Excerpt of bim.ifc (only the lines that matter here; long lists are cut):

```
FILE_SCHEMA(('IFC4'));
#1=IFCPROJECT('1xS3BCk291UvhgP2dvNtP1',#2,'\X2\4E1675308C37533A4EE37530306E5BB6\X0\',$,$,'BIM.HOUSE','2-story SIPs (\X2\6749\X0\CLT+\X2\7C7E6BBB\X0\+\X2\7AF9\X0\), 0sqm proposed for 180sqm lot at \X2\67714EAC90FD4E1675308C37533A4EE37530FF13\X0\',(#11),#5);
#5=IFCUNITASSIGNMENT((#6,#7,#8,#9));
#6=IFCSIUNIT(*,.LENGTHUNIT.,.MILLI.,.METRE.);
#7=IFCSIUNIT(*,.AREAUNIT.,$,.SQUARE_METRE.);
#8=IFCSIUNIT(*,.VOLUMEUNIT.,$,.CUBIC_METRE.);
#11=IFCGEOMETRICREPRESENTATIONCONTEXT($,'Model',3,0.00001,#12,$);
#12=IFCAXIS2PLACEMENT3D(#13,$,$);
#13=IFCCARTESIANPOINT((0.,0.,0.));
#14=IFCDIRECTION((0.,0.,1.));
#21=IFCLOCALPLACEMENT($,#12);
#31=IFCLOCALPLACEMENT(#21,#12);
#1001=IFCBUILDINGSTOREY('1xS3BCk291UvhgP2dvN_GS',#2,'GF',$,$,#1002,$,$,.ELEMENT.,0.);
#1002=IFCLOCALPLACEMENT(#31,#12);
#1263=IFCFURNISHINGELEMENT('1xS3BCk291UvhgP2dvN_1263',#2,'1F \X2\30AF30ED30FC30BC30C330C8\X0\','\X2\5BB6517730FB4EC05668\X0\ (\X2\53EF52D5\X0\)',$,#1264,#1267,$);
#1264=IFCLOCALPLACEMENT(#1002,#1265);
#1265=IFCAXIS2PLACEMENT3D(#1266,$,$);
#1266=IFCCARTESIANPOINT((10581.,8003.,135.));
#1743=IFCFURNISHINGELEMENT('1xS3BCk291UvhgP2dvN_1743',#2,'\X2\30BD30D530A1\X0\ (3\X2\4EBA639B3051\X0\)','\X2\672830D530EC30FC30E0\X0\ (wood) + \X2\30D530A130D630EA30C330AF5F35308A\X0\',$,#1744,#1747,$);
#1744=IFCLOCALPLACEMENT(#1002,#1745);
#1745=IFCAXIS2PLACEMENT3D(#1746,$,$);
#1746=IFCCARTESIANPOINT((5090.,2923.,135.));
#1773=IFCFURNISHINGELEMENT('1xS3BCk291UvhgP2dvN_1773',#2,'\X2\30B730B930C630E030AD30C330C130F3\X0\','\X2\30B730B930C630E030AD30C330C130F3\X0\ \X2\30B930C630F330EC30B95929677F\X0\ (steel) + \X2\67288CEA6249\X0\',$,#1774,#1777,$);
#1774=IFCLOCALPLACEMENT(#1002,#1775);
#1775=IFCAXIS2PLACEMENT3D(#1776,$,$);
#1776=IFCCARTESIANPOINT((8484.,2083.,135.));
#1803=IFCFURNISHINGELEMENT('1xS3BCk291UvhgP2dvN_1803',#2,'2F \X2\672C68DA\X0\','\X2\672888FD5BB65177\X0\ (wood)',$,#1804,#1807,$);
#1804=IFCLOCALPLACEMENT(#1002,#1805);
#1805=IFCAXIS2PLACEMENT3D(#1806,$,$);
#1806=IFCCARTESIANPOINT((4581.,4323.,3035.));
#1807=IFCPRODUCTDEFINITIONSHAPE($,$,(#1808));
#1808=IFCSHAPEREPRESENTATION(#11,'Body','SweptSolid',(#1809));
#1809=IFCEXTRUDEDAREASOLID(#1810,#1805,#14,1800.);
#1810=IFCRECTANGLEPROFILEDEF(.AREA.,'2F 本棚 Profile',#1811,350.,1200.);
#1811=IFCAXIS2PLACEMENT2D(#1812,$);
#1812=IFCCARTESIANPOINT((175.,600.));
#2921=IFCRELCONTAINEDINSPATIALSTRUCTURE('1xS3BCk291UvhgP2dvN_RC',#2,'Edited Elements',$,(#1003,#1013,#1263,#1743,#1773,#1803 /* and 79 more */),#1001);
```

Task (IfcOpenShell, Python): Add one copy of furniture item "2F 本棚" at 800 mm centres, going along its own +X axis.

```python
import ifcopenshell
import ifcopenshell.api.geometry
import ifcopenshell.api.root
import ifcopenshell.util.element
import ifcopenshell.util.placement

model = ifcopenshell.open("bim.ifc")


def reuse_history(source, copy):
    """copy_class also copies each property set's owner history, people and application; keep the originals."""
    for rel in copy.IsDefinedBy:
        if rel.is_a("IfcRelDefinesByProperties") and (history := rel.RelatingPropertyDefinition.OwnerHistory):
            rel.RelatingPropertyDefinition.OwnerHistory = source.OwnerHistory
            ifcopenshell.util.element.remove_deep2(model, history)


source = model.by_id(1803)
base = ifcopenshell.util.placement.get_local_placement(source.ObjectPlacement)
step = base[:3, 0] * 800.0

for i in range(1, 2):
    copy = ifcopenshell.api.root.copy_class(model, product=source)
    copy.Representation = ifcopenshell.util.element.copy_deep(
        model, source.Representation, exclude=["IfcGeometricRepresentationContext", "IfcRepresentationMap"]
    )
    reuse_history(source, copy)
    matrix = base.copy()
    matrix[:3, 3] += i * step
    print("added at", matrix[:3, 3].round(3) + 0.0)
    ifcopenshell.api.geometry.edit_object_placement(model, product=copy, matrix=matrix, is_si=False)

model.write("bim_edited.ifc")
```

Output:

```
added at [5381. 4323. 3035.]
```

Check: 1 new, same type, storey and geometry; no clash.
